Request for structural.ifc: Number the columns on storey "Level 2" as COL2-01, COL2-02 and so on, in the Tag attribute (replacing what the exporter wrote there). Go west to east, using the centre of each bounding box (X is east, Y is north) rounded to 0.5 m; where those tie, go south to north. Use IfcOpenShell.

First a look at what the model holds.

```python
import ifcopenshell
import ifcopenshell.util.element
import ifcopenshell.util.placement

model = ifcopenshell.open("structural.ifc")
print(model.schema)
storey = next(s for s in model.by_type("IfcBuildingStorey") if s.Name == "Level 2")
columns = [e for e in ifcopenshell.util.element.get_decomposition(storey) if e.is_a("IfcColumn")]
for e in sorted(columns, key=lambda e: e.id()):
    origin = ifcopenshell.util.placement.get_local_placement(e.ObjectPlacement)[:3, 3]
    print(e.id(), e.Tag, e.Name, origin.round(2) + 0.0, sep=" | ")
```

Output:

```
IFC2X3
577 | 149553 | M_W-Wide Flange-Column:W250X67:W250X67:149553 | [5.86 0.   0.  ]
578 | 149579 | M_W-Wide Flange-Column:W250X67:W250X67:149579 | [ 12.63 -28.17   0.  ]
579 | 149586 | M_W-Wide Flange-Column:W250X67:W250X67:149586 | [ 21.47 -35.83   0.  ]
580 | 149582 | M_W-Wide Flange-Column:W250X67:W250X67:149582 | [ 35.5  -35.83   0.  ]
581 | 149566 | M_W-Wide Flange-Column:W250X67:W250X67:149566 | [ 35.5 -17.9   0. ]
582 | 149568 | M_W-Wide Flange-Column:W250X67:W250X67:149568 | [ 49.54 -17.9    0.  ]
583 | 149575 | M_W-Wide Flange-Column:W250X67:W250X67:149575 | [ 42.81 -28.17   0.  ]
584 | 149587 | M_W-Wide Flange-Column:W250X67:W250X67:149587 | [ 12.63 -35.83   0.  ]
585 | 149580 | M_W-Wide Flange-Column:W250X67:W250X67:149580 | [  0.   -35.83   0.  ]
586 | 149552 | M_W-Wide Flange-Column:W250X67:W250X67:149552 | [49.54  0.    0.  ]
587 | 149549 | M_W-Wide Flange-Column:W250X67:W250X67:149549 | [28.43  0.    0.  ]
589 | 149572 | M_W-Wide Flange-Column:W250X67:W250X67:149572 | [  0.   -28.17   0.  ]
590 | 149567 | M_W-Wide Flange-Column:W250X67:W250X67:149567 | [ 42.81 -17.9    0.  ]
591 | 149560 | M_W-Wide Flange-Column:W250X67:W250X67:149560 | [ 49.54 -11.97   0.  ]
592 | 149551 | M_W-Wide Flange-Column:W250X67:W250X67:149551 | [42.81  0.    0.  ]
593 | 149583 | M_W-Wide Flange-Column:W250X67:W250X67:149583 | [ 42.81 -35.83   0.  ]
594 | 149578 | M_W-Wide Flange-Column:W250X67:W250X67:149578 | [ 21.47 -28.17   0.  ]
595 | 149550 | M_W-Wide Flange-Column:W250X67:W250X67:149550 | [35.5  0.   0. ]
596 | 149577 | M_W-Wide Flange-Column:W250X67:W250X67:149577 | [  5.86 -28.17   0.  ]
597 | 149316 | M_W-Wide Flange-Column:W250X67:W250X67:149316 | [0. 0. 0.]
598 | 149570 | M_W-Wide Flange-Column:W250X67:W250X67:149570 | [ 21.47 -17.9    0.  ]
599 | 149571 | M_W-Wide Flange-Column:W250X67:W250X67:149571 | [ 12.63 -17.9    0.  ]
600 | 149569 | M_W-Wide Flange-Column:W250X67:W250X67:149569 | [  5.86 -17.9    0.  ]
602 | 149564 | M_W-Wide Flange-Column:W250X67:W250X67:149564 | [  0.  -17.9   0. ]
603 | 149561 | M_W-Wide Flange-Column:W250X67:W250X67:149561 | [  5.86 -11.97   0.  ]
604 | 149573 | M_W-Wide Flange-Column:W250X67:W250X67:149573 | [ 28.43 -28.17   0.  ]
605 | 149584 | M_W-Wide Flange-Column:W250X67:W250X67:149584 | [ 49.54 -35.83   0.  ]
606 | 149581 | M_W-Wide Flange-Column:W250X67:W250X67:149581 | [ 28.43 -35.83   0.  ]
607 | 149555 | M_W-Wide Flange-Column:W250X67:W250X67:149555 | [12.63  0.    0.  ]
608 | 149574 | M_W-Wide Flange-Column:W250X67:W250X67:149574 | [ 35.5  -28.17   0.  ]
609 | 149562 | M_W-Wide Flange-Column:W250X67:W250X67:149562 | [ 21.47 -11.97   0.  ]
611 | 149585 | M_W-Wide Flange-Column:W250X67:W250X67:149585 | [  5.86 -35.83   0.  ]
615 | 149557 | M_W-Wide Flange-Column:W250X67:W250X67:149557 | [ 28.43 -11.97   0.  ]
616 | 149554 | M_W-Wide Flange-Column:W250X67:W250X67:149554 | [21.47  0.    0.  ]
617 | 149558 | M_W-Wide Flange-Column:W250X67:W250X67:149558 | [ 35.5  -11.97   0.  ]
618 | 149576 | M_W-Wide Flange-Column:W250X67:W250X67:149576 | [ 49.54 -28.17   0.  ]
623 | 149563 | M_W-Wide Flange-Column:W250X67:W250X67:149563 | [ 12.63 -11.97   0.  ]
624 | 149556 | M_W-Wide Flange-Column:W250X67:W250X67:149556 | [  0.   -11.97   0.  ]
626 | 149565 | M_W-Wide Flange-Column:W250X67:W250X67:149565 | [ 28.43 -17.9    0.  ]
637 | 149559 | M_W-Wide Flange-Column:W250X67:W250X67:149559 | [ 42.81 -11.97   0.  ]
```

```python
import ifcopenshell
import ifcopenshell.geom
import ifcopenshell.util.element
import ifcopenshell.util.shape

model = ifcopenshell.open("structural.ifc")
settings = ifcopenshell.geom.settings()
settings.set("use-world-coords", True)


def centre(element):
    shape = ifcopenshell.geom.create_shape(settings, element)
    return ifcopenshell.util.shape.get_bbox_centroid(shape.geometry)


storey = next(s for s in model.by_type("IfcBuildingStorey") if s.Name == "Level 2")
columns = [e for e in ifcopenshell.util.element.get_decomposition(storey) if e.is_a("IfcColumn")]

# Insertion points can sit at a corner or the storey origin, so sort by the geometry (in metres).
centres = {e: centre(e) for e in columns}
columns.sort(key=lambda e: (round(centres[e][0] / 0.5), centres[e][1]))

for i, e in enumerate(columns, start=1):
    number = f"COL2-{i:02d}"
    e.Tag = number
    print(e.id(), number)

model.write("structural_edited.ifc")
```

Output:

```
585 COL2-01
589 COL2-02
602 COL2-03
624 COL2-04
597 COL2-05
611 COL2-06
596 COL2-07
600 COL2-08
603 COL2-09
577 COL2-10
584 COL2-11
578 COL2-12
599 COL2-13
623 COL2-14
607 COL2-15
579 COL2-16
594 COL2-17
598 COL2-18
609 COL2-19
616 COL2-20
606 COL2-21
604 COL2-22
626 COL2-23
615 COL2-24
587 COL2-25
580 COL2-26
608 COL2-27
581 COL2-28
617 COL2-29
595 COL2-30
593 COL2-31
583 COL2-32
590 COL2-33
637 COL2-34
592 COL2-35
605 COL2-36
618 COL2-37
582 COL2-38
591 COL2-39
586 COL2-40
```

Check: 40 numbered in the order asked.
